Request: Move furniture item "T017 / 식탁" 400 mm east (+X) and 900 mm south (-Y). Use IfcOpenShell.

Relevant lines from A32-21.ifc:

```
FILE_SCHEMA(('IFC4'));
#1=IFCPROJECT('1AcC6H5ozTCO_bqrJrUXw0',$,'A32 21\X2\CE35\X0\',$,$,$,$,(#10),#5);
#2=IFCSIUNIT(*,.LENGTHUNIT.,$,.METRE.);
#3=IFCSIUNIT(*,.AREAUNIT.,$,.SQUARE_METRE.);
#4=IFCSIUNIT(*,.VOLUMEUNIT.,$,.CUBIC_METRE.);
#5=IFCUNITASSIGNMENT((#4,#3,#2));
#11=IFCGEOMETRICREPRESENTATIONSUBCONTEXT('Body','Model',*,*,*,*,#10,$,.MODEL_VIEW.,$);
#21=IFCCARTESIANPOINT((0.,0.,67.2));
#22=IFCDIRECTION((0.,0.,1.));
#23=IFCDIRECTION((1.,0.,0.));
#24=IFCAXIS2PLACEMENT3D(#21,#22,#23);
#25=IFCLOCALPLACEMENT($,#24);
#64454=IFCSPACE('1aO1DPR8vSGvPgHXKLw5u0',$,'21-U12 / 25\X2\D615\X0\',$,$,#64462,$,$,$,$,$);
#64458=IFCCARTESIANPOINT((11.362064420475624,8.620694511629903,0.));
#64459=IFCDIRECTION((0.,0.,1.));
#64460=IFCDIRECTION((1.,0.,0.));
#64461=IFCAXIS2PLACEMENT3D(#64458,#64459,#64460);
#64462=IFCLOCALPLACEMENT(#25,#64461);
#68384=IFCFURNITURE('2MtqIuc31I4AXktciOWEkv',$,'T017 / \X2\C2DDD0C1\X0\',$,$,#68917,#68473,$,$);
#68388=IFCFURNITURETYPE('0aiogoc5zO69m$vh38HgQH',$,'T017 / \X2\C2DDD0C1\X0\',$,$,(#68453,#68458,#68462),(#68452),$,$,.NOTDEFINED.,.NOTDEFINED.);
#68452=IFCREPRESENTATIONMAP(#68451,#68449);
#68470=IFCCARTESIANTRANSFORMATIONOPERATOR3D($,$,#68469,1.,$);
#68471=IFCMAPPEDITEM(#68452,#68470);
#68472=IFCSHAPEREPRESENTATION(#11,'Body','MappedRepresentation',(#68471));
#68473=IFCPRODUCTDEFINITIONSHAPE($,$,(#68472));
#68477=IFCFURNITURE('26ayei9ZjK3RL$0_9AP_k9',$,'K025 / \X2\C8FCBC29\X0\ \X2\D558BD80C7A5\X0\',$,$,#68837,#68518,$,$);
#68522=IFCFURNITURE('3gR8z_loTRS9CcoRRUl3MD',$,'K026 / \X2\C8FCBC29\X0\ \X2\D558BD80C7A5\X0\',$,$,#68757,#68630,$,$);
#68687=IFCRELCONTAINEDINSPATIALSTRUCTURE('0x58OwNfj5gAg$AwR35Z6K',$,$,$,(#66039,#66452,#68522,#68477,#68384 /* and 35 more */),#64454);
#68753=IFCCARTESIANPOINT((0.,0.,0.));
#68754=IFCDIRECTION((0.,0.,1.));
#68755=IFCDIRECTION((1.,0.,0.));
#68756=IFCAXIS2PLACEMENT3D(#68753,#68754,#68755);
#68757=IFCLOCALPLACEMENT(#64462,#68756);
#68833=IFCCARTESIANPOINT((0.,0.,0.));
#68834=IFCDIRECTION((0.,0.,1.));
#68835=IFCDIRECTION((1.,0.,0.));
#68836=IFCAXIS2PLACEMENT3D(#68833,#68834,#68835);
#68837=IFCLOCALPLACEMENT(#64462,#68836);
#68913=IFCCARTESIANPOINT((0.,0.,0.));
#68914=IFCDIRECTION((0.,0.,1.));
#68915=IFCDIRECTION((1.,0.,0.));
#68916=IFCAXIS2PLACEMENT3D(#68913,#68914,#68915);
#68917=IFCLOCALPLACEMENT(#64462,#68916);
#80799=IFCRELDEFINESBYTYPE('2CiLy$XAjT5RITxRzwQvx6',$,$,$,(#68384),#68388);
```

```python
import ifcopenshell
import ifcopenshell.api.geometry
import ifcopenshell.util.placement
import ifcopenshell.util.unit

model = ifcopenshell.open("A32-21.ifc")
unit_scale = ifcopenshell.util.unit.calculate_unit_scale(model)

item = model.by_guid("2MtqIuc31I4AXktciOWEkv")
matrix = ifcopenshell.util.placement.get_local_placement(item.ObjectPlacement)
matrix[0, 3] += 0.4 / unit_scale
matrix[1, 3] -= 0.9 / unit_scale
ifcopenshell.api.geometry.edit_object_placement(model, product=item, matrix=matrix, is_si=False)

print(ifcopenshell.util.placement.get_local_placement(item.ObjectPlacement).round(3) + 0.0)

model.write("A32-21_rev.ifc")
```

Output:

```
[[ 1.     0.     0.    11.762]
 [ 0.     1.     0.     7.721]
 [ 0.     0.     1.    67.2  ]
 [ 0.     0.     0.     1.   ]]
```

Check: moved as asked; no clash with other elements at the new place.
